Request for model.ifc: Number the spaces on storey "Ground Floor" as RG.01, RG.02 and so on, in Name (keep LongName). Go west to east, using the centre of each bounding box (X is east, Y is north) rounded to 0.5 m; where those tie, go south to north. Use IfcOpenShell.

First a look at what the model holds.

```python
import ifcopenshell
import ifcopenshell.util.element
import ifcopenshell.util.placement

model = ifcopenshell.open("model.ifc")
print(model.schema)
storey = next(s for s in model.by_type("IfcBuildingStorey") if s.Name == "Ground Floor")
spaces = [e for e in ifcopenshell.util.element.get_decomposition(storey) if e.is_a("IfcSpace")]
for e in sorted(spaces, key=lambda e: e.id()):
    origin = ifcopenshell.util.placement.get_local_placement(e.ObjectPlacement)[:3, 3]
    print(e.id(), e.Name, e.LongName, origin.round(2) + 0.0, sep=" | ")
```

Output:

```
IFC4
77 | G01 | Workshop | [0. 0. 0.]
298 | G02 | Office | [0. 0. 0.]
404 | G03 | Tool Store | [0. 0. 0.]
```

```python
import ifcopenshell
import ifcopenshell.geom
import ifcopenshell.util.element
import ifcopenshell.util.shape

model = ifcopenshell.open("model.ifc")
settings = ifcopenshell.geom.settings()
settings.set("use-world-coords", True)


def centre(element):
    shape = ifcopenshell.geom.create_shape(settings, element)
    return ifcopenshell.util.shape.get_bbox_centroid(shape.geometry)


storey = next(s for s in model.by_type("IfcBuildingStorey") if s.Name == "Ground Floor")
spaces = [e for e in ifcopenshell.util.element.get_decomposition(storey) if e.is_a("IfcSpace")]

# Insertion points can sit at a corner or the storey origin, so sort by the geometry (in metres).
centres = {e: centre(e) for e in spaces}
spaces.sort(key=lambda e: (round(centres[e][0] / 0.5), centres[e][1]))

for i, e in enumerate(spaces, start=1):
    number = f"RG.{i:02d}"
    e.Name = number
    print(e.id(), number)

model.write("model_updated.ifc")
```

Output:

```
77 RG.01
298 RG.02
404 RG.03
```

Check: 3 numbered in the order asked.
